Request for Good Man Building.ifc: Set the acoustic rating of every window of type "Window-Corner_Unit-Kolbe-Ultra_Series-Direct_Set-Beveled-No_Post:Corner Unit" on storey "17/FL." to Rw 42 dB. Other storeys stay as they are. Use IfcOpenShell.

First a look at what the model holds.

```python
import ifcopenshell
import ifcopenshell.util.element

model = ifcopenshell.open("Good Man Building.ifc")
print(model.schema)
storey = next(s for s in model.by_type("IfcBuildingStorey") if s.Name == "17/FL.")
windows = [e for e in ifcopenshell.util.element.get_decomposition(storey) if e.is_a("IfcWindow")]
seen = {}
for e in windows:
    element_type = ifcopenshell.util.element.get_type(e)
    key = (element_type.Name if element_type != e and element_type else None, ifcopenshell.util.element.get_pset(e, "Pset_WindowCommon", "AcousticRating"))
    seen[key] = seen.get(key, 0) + 1
for (name, value), count in sorted(seen.items(), key=str):
    print(count, "x", name, "|", value)
```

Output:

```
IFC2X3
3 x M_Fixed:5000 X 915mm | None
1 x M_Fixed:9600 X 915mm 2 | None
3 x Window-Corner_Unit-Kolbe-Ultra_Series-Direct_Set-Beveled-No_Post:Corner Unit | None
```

```python
import ifcopenshell
import ifcopenshell.api.pset
import ifcopenshell.util.element

model = ifcopenshell.open("Good Man Building.ifc")

storey = next(s for s in model.by_type("IfcBuildingStorey") if s.Name == "17/FL.")
windows = [e for e in ifcopenshell.util.element.get_decomposition(storey) if e.is_a("IfcWindow")]

count = 0
for e in windows:
    element_type = ifcopenshell.util.element.get_type(e)
    if element_type in (None, e) or element_type.Name != "Window-Corner_Unit-Kolbe-Ultra_Series-Direct_Set-Beveled-No_Post:Corner Unit":
        continue
    # add_pset returns the element's existing set when there is one.
    pset = ifcopenshell.api.pset.add_pset(model, product=e, name="Pset_WindowCommon")
    ifcopenshell.api.pset.edit_pset(model, pset=pset, properties={"AcousticRating": "Rw 42 dB"})
    count += 1

print(count, "windows updated")

model.write("Good Man Building_updated.ifc")
```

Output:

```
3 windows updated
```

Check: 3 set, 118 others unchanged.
